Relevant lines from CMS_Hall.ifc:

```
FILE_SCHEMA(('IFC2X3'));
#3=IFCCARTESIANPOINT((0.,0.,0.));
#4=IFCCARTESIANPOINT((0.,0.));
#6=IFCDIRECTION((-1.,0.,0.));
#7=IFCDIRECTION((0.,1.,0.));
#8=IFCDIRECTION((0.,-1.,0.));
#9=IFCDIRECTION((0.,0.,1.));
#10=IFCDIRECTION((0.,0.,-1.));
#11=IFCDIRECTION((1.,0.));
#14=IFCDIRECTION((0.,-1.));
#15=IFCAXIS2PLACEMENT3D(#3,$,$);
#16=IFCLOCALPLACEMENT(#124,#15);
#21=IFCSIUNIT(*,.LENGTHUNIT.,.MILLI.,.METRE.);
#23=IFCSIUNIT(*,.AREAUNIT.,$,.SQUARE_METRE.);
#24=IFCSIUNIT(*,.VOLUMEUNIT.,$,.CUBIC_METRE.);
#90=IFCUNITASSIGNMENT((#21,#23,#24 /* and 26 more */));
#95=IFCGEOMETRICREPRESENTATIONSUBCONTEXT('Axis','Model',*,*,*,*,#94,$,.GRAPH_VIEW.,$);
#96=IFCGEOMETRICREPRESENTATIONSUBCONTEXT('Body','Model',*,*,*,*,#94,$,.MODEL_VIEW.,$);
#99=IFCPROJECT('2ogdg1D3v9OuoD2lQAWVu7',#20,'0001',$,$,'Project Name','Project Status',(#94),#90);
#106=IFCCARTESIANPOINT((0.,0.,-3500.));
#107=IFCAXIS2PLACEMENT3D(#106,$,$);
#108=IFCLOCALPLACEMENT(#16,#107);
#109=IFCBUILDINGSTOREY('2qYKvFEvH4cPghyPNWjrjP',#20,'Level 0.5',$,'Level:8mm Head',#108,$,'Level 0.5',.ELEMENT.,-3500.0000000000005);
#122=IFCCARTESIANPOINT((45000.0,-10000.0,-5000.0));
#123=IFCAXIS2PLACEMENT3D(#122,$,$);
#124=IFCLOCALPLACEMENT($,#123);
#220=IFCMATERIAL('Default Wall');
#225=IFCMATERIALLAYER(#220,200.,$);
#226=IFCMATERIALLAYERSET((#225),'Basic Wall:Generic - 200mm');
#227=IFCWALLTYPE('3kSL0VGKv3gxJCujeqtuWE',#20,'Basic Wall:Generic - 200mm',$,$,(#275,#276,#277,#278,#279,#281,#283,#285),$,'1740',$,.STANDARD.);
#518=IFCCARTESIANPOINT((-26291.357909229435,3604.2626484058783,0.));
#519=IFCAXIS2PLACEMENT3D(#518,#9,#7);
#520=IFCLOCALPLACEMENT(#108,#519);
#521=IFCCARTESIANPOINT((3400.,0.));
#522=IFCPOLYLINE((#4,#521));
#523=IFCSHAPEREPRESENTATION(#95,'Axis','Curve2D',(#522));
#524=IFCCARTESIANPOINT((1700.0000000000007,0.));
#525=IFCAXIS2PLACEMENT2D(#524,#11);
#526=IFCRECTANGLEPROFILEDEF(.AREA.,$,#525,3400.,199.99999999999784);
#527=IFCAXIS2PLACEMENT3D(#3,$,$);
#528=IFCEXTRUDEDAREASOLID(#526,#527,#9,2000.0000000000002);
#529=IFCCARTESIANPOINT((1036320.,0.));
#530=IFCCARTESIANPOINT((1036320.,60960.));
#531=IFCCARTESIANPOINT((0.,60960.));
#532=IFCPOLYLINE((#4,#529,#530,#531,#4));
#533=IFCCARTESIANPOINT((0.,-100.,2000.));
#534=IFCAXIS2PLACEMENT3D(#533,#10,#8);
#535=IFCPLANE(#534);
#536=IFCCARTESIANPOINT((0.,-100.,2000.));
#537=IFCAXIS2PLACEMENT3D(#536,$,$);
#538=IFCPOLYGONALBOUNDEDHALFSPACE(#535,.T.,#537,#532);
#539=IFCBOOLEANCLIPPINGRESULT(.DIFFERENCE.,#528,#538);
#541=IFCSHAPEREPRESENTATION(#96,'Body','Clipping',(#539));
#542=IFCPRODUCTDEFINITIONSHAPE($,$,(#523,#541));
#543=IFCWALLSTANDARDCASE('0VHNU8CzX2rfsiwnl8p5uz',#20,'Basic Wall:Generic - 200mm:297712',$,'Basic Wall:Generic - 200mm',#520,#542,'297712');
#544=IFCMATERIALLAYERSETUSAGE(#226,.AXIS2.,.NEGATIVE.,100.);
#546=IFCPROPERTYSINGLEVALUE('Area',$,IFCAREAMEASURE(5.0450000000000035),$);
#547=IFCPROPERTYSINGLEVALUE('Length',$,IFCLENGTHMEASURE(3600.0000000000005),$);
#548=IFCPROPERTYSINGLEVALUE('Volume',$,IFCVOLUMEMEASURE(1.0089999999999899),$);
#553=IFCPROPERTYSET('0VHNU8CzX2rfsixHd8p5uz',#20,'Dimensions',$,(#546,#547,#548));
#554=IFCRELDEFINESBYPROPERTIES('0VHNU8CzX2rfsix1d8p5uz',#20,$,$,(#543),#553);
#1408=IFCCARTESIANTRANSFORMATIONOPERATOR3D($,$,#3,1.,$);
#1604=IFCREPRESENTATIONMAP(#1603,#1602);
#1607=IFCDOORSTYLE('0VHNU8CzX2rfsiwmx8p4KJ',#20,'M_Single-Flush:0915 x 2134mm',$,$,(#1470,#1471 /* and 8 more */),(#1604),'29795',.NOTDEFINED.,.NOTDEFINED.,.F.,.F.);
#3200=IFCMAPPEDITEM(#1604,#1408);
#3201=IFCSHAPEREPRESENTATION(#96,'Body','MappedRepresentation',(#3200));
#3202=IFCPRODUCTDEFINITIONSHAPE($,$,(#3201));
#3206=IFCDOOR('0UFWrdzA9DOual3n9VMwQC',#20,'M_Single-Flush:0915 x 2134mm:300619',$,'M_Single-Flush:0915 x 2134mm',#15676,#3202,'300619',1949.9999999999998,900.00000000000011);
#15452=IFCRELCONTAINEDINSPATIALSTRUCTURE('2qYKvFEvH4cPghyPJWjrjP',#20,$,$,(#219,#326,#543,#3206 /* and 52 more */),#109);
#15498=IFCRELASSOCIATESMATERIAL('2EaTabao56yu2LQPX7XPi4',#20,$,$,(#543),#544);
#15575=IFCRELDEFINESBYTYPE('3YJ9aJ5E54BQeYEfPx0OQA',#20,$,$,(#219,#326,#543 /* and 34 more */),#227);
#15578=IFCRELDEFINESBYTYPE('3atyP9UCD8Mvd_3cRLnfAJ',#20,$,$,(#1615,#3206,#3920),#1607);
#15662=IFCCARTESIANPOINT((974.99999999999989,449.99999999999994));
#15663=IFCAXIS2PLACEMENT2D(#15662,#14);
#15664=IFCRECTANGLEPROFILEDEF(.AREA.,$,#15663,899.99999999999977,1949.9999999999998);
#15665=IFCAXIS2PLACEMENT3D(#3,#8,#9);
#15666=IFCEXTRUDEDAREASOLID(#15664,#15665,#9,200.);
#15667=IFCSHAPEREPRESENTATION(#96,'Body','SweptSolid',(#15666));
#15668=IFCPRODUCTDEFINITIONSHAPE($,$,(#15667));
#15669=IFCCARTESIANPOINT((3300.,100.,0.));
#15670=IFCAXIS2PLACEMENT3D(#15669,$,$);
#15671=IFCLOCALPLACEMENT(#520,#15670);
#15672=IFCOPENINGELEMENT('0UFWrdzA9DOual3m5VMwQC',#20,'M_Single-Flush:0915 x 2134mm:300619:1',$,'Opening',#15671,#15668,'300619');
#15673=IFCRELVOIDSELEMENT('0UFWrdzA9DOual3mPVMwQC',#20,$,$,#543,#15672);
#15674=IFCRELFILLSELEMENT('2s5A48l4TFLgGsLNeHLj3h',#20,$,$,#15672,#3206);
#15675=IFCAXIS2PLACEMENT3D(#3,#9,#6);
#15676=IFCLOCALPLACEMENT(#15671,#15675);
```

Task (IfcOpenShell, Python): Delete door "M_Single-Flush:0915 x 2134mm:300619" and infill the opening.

```python
import ifcopenshell
import ifcopenshell.api.feature
import ifcopenshell.api.pset
import ifcopenshell.api.root
import ifcopenshell.geom
import ifcopenshell.util.element
import ifcopenshell.util.shape
import ifcopenshell.util.unit

model = ifcopenshell.open("CMS_Hall.ifc")
area_scale = ifcopenshell.util.unit.calculate_unit_scale(model, "AREAUNIT")
volume_scale = ifcopenshell.util.unit.calculate_unit_scale(model, "VOLUMEUNIT")
settings = ifcopenshell.geom.settings()


def volume(element):
    """Net volume in cubic metres, openings subtracted."""
    shape = ifcopenshell.geom.create_shape(settings, element)
    return ifcopenshell.util.shape.get_volume(shape.geometry)


door = model.by_id(3206)
opening = door.FillsVoids[0].RelatingOpeningElement
wall = opening.VoidsElements[0].RelatingBuildingElement
before = volume(wall)

ifcopenshell.api.root.remove_product(model, product=door)
ifcopenshell.api.feature.remove_feature(model, feature=opening)

after = volume(wall)
thickness = 0.2  # wall thickness in metres

# Update the wall's stored quantities.
pset = model.by_id(ifcopenshell.util.element.get_pset(wall, "Dimensions", should_inherit=False)["id"])
ifcopenshell.api.pset.edit_pset(model, pset=pset, properties={
    "Area": model.create_entity("IfcAreaMeasure", after / thickness / area_scale),
    "Volume": model.create_entity("IfcVolumeMeasure", after / volume_scale),
})

print(f"wall volume {before:.3f} -> {after:.3f} m3")

model.write("CMS_Hall_v2.ifc")
```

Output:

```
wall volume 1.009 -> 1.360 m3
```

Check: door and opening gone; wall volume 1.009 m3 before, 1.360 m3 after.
